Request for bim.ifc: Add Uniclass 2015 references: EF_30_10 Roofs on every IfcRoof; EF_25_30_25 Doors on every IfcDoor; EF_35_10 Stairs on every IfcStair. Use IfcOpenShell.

First a look at what the model holds.

```python
import ifcopenshell

model = ifcopenshell.open("bim.ifc")
print(model.schema)
print("classifications:", [c.Name for c in model.by_type("IfcClassification")])
for ifc_class in ("IfcDoor", "IfcRoof", "IfcStair", "IfcWall", "IfcWindow"):
    print(ifc_class, len(model.by_type(ifc_class)))
```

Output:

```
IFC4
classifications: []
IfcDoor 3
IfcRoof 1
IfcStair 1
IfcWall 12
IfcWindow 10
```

```python
import ifcopenshell
import ifcopenshell.api.classification

model = ifcopenshell.open("bim.ifc")

system = ifcopenshell.api.classification.add_classification(model, classification="Uniclass 2015")

codes = {
    "IfcRoof": ("EF_30_10", "Roofs"),
    "IfcDoor": ("EF_25_30_25", "Doors"),
    "IfcStair": ("EF_35_10", "Stairs"),
}
for ifc_class, (code, name) in codes.items():
    products = model.by_type(ifc_class)
    ifcopenshell.api.classification.add_reference(
        model, products=products, classification=system, identification=code, name=name
    )
    print(code, len(products))

model.write("bim_v2.ifc")
```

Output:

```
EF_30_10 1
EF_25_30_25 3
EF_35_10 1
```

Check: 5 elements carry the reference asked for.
